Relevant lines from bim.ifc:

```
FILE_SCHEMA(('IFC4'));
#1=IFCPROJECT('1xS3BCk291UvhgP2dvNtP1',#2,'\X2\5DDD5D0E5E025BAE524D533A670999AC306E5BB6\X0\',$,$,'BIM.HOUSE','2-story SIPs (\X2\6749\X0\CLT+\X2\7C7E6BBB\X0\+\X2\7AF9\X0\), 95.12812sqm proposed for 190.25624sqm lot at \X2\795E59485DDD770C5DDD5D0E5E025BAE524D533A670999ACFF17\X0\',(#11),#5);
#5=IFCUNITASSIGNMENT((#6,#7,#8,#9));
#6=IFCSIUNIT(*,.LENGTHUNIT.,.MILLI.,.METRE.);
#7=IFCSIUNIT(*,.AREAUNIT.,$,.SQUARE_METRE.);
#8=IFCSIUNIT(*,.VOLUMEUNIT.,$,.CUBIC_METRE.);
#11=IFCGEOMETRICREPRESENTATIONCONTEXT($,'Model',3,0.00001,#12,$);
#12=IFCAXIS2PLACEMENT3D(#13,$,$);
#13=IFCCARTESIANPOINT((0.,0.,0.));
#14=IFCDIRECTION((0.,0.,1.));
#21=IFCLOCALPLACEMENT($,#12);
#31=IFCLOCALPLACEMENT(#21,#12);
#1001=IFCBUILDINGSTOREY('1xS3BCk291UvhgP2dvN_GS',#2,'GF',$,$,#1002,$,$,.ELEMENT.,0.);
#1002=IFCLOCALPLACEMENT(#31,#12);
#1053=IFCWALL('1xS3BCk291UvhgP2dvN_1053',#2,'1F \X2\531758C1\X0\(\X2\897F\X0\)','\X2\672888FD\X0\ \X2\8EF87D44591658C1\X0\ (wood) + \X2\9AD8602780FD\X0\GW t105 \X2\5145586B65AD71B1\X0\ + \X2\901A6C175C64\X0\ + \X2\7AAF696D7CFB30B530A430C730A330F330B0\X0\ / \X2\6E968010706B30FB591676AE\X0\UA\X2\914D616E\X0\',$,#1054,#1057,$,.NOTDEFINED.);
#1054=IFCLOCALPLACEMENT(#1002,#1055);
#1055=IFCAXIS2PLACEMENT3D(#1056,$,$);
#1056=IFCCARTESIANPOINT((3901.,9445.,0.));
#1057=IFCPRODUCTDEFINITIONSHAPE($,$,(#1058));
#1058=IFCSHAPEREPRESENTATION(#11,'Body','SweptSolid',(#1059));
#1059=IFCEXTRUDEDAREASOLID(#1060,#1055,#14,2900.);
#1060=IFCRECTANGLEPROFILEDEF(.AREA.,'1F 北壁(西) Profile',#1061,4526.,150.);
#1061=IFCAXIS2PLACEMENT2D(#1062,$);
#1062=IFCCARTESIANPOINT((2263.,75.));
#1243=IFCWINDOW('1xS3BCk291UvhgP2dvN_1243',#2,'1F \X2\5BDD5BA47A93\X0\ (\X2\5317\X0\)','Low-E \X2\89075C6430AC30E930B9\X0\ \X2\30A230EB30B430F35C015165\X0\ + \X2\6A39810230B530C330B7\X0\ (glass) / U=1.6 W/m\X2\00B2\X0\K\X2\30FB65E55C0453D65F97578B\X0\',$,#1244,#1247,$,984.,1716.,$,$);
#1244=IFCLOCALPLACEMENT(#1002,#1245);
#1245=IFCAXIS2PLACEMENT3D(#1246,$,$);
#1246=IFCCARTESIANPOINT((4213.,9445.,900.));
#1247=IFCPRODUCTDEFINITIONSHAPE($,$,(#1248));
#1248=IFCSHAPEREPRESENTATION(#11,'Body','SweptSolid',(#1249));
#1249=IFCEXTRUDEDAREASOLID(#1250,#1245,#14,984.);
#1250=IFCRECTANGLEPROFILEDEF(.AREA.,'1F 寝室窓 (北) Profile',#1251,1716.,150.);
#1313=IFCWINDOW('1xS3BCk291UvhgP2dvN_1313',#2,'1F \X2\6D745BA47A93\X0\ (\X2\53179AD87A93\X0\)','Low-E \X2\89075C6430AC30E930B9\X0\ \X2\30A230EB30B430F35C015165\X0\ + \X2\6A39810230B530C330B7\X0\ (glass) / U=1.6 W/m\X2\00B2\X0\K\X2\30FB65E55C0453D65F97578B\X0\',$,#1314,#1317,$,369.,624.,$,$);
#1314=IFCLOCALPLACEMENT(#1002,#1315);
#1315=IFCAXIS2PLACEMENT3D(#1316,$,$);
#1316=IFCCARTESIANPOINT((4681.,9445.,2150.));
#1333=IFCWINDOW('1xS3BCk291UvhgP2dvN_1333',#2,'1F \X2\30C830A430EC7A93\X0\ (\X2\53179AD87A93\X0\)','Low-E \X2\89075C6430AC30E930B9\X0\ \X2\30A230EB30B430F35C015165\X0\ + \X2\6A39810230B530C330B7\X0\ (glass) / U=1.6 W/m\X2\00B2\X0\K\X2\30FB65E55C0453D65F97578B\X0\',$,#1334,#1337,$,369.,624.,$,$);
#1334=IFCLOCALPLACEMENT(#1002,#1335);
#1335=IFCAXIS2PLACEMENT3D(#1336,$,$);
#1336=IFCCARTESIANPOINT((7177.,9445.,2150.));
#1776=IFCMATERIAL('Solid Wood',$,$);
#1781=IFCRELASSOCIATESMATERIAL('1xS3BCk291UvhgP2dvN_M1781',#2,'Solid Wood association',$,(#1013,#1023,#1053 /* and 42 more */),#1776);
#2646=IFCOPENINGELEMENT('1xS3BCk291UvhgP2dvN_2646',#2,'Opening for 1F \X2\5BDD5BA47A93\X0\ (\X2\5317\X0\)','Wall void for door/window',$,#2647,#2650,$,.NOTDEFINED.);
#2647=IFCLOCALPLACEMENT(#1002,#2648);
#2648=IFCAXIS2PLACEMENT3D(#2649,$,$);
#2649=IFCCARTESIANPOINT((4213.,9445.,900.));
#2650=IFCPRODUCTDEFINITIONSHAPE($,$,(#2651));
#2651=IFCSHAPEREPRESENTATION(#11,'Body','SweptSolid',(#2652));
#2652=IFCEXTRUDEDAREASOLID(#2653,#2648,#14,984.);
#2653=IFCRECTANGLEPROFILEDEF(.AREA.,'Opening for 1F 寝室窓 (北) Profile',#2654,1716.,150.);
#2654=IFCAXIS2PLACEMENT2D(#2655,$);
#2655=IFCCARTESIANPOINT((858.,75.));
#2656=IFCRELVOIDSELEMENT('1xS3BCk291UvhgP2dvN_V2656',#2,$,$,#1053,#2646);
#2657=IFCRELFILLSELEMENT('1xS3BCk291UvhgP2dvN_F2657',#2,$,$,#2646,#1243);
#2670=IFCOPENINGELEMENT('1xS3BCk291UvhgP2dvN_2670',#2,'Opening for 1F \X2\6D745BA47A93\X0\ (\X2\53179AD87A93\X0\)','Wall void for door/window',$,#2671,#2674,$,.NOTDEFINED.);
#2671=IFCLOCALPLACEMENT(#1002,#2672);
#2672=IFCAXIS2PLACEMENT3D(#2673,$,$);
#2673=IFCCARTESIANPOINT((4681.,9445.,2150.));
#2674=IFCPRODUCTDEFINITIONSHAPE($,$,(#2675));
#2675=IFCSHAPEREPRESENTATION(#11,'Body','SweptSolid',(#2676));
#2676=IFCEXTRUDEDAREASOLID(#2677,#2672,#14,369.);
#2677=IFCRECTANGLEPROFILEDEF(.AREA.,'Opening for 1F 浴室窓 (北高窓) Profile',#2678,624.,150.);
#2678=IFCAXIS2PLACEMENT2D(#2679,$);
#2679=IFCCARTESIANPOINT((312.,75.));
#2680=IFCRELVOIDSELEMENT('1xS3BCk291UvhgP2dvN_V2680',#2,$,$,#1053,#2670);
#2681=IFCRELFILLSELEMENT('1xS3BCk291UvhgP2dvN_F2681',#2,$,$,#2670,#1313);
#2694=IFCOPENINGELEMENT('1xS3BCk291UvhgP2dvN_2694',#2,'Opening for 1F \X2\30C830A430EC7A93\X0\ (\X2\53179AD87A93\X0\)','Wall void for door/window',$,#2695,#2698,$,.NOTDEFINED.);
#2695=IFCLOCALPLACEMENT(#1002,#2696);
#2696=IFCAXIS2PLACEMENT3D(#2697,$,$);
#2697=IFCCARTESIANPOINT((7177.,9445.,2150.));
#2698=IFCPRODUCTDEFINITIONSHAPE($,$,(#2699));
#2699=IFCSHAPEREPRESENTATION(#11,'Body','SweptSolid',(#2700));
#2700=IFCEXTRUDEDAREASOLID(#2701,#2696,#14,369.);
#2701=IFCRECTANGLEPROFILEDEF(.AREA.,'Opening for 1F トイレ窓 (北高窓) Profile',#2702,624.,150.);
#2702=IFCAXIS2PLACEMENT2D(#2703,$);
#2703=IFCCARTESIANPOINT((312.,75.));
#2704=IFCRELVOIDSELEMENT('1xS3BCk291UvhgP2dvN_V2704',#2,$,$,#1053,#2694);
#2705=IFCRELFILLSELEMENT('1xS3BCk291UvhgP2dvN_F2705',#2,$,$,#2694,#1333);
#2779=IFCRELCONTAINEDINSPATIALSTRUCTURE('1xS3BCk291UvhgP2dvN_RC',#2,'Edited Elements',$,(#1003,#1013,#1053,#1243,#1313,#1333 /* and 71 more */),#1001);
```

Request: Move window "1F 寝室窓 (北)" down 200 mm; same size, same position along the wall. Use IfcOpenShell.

```python
import numpy as np
import ifcopenshell
import ifcopenshell.api.geometry
import ifcopenshell.util.placement
import ifcopenshell.util.unit

model = ifcopenshell.open("bim.ifc")
unit_scale = ifcopenshell.util.unit.calculate_unit_scale(model)

window = model.by_id(1243)
opening = window.FillsVoids[0].RelatingOpeningElement
dz = -200.0

shift = np.array([0.0, 0.0, dz])
# The window is not placed relative to its opening, so move both.
for product in (opening, window):
    matrix = ifcopenshell.util.placement.get_local_placement(product.ObjectPlacement)
    matrix[:3, 3] += shift
    ifcopenshell.api.geometry.edit_object_placement(model, product=product, matrix=matrix, is_si=False)

print(f"moved by {dz * unit_scale:+.3f} m")

model.write("bim_rev.ifc")
```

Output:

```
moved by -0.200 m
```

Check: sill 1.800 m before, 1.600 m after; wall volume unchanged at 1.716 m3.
